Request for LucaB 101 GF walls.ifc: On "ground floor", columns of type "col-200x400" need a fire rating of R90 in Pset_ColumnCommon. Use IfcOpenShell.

First a look at what the model holds.

```python
import ifcopenshell
import ifcopenshell.util.element

model = ifcopenshell.open("LucaB 101 GF walls.ifc")
print(model.schema)
storey = next(s for s in model.by_type("IfcBuildingStorey") if s.Name == "ground floor")
columns = [e for e in ifcopenshell.util.element.get_decomposition(storey) if e.is_a("IfcColumn")]
seen = {}
for e in columns:
    element_type = ifcopenshell.util.element.get_type(e)
    key = (element_type.Name if element_type != e and element_type else None, ifcopenshell.util.element.get_pset(e, "Pset_ColumnCommon", "FireRating"))
    seen[key] = seen.get(key, 0) + 1
for (name, value), count in sorted(seen.items(), key=str):
    print(count, "x", name, "|", value)
```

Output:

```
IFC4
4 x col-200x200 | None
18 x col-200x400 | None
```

```python
import ifcopenshell
import ifcopenshell.api.pset
import ifcopenshell.util.element

model = ifcopenshell.open("LucaB 101 GF walls.ifc")

storey = next(s for s in model.by_type("IfcBuildingStorey") if s.Name == "ground floor")
columns = [e for e in ifcopenshell.util.element.get_decomposition(storey) if e.is_a("IfcColumn")]

count = 0
for e in columns:
    element_type = ifcopenshell.util.element.get_type(e)
    if element_type in (None, e) or element_type.Name != "col-200x400":
        continue
    # add_pset returns the element's existing set when there is one.
    pset = ifcopenshell.api.pset.add_pset(model, product=e, name="Pset_ColumnCommon")
    ifcopenshell.api.pset.edit_pset(model, pset=pset, properties={"FireRating": "R90"})
    count += 1

print(count, "columns updated")

model.write("LucaB 101 GF walls_edited.ifc")
```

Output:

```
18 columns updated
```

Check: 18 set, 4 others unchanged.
